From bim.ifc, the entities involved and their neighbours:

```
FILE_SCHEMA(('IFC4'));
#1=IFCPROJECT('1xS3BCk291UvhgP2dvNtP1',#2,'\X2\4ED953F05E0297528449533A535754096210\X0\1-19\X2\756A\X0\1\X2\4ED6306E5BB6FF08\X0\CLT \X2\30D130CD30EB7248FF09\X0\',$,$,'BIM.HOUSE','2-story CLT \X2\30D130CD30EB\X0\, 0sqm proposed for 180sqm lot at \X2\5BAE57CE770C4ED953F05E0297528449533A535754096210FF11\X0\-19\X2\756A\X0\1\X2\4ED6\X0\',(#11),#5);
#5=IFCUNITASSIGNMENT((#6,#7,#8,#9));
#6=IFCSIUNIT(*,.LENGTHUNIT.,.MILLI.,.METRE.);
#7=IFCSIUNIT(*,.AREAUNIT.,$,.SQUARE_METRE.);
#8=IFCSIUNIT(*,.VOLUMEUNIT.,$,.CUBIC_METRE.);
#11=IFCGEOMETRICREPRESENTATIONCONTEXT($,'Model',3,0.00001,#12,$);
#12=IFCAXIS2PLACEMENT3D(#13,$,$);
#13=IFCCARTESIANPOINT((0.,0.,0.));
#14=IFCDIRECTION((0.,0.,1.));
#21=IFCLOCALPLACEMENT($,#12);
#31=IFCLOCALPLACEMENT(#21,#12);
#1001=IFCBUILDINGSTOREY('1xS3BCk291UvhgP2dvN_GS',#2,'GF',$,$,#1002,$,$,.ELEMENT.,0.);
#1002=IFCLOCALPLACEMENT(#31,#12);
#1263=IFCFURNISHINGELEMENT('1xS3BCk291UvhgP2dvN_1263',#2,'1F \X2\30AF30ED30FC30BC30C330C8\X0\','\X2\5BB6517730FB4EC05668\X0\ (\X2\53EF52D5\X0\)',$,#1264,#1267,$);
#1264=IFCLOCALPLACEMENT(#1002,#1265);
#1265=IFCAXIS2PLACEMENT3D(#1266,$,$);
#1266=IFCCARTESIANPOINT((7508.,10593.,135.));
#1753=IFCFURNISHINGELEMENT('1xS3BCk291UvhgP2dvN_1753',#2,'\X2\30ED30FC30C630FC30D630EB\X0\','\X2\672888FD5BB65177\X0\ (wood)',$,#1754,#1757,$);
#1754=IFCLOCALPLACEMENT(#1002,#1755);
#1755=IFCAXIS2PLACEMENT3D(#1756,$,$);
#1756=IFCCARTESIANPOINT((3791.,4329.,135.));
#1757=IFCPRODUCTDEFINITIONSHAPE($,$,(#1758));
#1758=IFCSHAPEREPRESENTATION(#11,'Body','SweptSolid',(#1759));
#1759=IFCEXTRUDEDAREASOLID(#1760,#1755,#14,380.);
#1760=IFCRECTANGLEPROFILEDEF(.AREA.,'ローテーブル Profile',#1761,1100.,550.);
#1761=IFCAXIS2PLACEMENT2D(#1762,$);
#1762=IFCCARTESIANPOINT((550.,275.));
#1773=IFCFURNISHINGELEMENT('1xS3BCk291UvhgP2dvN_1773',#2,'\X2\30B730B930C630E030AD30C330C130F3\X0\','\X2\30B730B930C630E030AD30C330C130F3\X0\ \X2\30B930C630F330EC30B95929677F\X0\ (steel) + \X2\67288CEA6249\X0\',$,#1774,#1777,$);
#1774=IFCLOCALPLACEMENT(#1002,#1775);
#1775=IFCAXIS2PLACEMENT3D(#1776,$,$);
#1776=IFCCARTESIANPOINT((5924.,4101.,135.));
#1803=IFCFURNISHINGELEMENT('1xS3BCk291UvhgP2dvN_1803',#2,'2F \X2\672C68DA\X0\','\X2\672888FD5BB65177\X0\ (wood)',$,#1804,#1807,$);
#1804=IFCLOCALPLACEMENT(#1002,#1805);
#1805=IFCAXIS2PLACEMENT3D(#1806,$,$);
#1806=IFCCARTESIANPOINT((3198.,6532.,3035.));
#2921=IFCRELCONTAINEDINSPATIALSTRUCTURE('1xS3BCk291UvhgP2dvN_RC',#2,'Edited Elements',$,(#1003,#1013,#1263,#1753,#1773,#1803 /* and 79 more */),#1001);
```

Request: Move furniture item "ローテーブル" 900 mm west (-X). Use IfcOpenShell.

```python
import ifcopenshell
import ifcopenshell.api.geometry
import ifcopenshell.util.placement

model = ifcopenshell.open("bim.ifc")

item = model.by_guid("1xS3BCk291UvhgP2dvN_1753")
matrix = ifcopenshell.util.placement.get_local_placement(item.ObjectPlacement)
matrix[0, 3] -= 900.0
ifcopenshell.api.geometry.edit_object_placement(model, product=item, matrix=matrix, is_si=False)

print(ifcopenshell.util.placement.get_local_placement(item.ObjectPlacement).round(3) + 0.0)

model.write("bim-out.ifc")
```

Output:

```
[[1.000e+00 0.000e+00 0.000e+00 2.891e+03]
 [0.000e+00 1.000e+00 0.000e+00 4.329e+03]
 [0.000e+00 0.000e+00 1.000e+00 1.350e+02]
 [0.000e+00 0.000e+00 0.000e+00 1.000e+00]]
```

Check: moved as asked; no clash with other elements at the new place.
